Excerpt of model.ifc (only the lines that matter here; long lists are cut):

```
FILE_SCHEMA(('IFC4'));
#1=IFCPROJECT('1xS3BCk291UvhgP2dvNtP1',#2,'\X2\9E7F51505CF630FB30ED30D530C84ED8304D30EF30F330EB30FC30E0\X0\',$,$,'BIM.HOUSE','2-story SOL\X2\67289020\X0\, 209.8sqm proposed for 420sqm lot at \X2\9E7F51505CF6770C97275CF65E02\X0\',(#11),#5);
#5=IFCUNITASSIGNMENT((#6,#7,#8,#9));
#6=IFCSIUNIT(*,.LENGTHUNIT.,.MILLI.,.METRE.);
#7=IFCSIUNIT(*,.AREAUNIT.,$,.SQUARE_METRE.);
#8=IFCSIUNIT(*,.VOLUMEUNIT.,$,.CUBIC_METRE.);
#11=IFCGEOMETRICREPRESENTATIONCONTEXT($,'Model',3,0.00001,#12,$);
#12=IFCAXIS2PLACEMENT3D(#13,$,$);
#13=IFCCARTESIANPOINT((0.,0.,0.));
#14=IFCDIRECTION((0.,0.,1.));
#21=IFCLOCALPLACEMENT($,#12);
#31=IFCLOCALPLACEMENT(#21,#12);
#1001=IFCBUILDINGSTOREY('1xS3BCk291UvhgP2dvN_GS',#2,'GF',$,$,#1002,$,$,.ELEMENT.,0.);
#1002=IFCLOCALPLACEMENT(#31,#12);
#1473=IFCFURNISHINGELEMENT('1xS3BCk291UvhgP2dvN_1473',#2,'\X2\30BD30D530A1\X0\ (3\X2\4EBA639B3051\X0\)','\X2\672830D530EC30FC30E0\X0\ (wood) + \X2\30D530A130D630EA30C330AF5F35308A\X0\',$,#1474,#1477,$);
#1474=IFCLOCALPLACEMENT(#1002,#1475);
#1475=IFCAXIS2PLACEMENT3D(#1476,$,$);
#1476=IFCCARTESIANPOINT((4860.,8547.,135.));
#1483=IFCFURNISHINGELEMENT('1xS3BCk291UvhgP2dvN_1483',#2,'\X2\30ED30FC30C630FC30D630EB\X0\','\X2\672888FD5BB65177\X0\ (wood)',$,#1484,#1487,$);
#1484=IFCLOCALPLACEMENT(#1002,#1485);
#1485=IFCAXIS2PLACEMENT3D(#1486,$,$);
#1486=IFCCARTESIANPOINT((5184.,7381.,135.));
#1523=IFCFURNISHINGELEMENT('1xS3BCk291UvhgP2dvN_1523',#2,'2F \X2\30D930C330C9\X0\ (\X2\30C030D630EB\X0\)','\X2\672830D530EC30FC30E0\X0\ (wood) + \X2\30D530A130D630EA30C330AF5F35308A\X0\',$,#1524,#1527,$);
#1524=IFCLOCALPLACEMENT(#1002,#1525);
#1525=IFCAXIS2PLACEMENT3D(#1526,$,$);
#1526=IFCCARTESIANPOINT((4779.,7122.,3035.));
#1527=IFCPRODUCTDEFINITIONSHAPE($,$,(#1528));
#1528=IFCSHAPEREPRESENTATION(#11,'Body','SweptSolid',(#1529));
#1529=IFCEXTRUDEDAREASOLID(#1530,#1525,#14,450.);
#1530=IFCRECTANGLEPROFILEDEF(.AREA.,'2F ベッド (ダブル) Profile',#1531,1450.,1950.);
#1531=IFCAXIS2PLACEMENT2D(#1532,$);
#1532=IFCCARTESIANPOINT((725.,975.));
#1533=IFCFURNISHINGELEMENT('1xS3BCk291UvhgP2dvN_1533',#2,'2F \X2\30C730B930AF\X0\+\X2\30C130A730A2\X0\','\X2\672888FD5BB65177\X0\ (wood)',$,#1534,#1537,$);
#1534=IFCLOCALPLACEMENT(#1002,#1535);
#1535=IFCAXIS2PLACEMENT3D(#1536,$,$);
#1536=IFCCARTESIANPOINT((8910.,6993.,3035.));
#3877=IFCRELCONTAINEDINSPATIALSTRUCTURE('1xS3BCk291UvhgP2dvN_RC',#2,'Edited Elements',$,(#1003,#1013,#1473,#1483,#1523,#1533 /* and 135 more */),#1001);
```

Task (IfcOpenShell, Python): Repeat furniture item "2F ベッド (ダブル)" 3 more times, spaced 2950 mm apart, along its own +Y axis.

```python
import ifcopenshell
import ifcopenshell.api.geometry
import ifcopenshell.api.root
import ifcopenshell.util.element
import ifcopenshell.util.placement

model = ifcopenshell.open("model.ifc")


def reuse_history(source, copy):
    """copy_class also copies each property set's owner history, people and application; keep the originals."""
    for rel in copy.IsDefinedBy:
        if rel.is_a("IfcRelDefinesByProperties") and (history := rel.RelatingPropertyDefinition.OwnerHistory):
            rel.RelatingPropertyDefinition.OwnerHistory = source.OwnerHistory
            ifcopenshell.util.element.remove_deep2(model, history)


source = model.by_guid("1xS3BCk291UvhgP2dvN_1523")
base = ifcopenshell.util.placement.get_local_placement(source.ObjectPlacement)
step = base[:3, 1] * 2950.0

for i in range(1, 4):
    copy = ifcopenshell.api.root.copy_class(model, product=source)
    copy.Representation = ifcopenshell.util.element.copy_deep(
        model, source.Representation, exclude=["IfcGeometricRepresentationContext", "IfcRepresentationMap"]
    )
    reuse_history(source, copy)
    matrix = base.copy()
    matrix[:3, 3] += i * step
    print("added at", matrix[:3, 3].round(3) + 0.0)
    ifcopenshell.api.geometry.edit_object_placement(model, product=copy, matrix=matrix, is_si=False)

model.write("model-out.ifc")
```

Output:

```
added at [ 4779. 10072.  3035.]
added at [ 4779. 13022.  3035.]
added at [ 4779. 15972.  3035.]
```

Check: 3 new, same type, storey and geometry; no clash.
